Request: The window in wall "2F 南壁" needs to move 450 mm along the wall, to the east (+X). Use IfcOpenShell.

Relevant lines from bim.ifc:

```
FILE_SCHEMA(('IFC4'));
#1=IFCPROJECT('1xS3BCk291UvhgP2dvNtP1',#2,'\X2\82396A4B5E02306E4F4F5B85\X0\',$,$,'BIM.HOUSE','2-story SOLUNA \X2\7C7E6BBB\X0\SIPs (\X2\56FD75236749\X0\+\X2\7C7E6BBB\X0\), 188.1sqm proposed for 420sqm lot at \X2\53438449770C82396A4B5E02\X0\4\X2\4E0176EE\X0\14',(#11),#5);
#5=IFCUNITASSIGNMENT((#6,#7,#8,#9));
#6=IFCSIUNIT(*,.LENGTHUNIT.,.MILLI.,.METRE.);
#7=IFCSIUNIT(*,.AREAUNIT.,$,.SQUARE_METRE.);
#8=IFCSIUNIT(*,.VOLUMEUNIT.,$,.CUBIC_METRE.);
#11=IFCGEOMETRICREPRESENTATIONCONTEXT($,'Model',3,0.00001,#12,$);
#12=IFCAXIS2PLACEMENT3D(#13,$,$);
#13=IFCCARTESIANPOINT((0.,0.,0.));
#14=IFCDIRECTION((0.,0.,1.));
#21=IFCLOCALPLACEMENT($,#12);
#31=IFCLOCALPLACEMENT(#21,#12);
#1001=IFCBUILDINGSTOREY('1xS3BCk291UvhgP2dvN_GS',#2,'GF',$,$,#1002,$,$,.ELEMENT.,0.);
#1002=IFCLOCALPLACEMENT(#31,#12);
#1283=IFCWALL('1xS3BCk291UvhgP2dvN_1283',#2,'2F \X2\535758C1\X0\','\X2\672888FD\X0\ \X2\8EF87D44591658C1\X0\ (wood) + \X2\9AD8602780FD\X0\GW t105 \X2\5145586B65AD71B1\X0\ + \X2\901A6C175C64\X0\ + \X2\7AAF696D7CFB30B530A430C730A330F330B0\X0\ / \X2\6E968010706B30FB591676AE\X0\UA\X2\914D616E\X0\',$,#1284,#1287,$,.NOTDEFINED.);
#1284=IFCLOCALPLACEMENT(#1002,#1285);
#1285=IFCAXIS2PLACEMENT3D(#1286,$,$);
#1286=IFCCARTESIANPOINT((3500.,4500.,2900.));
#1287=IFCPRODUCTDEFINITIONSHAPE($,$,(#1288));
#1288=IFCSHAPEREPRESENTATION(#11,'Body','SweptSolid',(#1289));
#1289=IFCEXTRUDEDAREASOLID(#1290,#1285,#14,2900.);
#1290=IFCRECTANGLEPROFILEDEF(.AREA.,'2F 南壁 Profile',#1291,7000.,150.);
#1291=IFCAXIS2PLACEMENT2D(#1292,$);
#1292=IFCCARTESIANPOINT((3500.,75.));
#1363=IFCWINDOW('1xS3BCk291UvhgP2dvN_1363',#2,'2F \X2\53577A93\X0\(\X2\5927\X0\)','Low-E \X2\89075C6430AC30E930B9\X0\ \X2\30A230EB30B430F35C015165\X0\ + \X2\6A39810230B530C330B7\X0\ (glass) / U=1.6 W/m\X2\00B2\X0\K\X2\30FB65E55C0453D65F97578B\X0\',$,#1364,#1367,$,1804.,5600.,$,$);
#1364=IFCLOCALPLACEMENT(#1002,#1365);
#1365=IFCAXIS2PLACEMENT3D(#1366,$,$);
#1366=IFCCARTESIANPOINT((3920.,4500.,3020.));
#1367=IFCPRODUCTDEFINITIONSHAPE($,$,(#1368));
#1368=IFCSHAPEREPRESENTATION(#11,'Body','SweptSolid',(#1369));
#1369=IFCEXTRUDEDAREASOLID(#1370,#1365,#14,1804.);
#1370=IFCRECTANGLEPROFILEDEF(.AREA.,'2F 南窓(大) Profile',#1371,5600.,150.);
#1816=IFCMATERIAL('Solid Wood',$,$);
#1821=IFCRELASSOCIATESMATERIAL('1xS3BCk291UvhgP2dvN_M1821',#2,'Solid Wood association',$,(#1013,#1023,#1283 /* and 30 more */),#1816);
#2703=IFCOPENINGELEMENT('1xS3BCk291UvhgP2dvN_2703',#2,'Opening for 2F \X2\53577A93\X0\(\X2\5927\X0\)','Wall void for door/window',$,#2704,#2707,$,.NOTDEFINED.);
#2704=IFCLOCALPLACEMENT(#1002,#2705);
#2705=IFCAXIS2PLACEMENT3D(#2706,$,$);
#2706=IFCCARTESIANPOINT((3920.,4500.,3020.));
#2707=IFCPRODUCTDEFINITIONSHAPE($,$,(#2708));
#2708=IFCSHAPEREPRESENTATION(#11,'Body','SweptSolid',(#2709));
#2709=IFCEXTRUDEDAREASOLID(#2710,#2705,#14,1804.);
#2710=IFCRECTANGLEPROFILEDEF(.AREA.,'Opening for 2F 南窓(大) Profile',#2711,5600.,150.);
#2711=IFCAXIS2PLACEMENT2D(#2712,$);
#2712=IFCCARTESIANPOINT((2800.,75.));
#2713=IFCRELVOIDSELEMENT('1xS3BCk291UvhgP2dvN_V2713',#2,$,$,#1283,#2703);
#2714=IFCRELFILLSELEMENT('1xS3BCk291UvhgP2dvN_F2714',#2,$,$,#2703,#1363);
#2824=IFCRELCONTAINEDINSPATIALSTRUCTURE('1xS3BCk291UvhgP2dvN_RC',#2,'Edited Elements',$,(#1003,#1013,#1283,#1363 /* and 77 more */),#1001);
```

```python
import ifcopenshell
import ifcopenshell.api.geometry
import ifcopenshell.util.placement
import ifcopenshell.util.unit

model = ifcopenshell.open("bim.ifc")
unit_scale = ifcopenshell.util.unit.calculate_unit_scale(model)

window = model.by_guid("1xS3BCk291UvhgP2dvN_1363")
opening = window.FillsVoids[0].RelatingOpeningElement
wall = opening.VoidsElements[0].RelatingBuildingElement

wall_matrix = ifcopenshell.util.placement.get_local_placement(wall.ObjectPlacement)
shift = wall_matrix[:3, 0] * 0.45 / unit_scale
before = ifcopenshell.util.placement.get_local_placement(window.ObjectPlacement)[:3, 3].copy()

# The window is not placed relative to its opening, so move both.
for product in (opening, window):
    matrix = ifcopenshell.util.placement.get_local_placement(product.ObjectPlacement)
    matrix[:3, 3] += shift
    ifcopenshell.api.geometry.edit_object_placement(model, product=product, matrix=matrix, is_si=False)

after = ifcopenshell.util.placement.get_local_placement(window.ObjectPlacement)[:3, 3]
print("window moved by", (after - before).round(3) + 0.0)

model.write("bim_updated.ifc")
```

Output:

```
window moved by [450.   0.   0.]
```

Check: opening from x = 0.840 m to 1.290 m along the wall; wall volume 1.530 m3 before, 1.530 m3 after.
